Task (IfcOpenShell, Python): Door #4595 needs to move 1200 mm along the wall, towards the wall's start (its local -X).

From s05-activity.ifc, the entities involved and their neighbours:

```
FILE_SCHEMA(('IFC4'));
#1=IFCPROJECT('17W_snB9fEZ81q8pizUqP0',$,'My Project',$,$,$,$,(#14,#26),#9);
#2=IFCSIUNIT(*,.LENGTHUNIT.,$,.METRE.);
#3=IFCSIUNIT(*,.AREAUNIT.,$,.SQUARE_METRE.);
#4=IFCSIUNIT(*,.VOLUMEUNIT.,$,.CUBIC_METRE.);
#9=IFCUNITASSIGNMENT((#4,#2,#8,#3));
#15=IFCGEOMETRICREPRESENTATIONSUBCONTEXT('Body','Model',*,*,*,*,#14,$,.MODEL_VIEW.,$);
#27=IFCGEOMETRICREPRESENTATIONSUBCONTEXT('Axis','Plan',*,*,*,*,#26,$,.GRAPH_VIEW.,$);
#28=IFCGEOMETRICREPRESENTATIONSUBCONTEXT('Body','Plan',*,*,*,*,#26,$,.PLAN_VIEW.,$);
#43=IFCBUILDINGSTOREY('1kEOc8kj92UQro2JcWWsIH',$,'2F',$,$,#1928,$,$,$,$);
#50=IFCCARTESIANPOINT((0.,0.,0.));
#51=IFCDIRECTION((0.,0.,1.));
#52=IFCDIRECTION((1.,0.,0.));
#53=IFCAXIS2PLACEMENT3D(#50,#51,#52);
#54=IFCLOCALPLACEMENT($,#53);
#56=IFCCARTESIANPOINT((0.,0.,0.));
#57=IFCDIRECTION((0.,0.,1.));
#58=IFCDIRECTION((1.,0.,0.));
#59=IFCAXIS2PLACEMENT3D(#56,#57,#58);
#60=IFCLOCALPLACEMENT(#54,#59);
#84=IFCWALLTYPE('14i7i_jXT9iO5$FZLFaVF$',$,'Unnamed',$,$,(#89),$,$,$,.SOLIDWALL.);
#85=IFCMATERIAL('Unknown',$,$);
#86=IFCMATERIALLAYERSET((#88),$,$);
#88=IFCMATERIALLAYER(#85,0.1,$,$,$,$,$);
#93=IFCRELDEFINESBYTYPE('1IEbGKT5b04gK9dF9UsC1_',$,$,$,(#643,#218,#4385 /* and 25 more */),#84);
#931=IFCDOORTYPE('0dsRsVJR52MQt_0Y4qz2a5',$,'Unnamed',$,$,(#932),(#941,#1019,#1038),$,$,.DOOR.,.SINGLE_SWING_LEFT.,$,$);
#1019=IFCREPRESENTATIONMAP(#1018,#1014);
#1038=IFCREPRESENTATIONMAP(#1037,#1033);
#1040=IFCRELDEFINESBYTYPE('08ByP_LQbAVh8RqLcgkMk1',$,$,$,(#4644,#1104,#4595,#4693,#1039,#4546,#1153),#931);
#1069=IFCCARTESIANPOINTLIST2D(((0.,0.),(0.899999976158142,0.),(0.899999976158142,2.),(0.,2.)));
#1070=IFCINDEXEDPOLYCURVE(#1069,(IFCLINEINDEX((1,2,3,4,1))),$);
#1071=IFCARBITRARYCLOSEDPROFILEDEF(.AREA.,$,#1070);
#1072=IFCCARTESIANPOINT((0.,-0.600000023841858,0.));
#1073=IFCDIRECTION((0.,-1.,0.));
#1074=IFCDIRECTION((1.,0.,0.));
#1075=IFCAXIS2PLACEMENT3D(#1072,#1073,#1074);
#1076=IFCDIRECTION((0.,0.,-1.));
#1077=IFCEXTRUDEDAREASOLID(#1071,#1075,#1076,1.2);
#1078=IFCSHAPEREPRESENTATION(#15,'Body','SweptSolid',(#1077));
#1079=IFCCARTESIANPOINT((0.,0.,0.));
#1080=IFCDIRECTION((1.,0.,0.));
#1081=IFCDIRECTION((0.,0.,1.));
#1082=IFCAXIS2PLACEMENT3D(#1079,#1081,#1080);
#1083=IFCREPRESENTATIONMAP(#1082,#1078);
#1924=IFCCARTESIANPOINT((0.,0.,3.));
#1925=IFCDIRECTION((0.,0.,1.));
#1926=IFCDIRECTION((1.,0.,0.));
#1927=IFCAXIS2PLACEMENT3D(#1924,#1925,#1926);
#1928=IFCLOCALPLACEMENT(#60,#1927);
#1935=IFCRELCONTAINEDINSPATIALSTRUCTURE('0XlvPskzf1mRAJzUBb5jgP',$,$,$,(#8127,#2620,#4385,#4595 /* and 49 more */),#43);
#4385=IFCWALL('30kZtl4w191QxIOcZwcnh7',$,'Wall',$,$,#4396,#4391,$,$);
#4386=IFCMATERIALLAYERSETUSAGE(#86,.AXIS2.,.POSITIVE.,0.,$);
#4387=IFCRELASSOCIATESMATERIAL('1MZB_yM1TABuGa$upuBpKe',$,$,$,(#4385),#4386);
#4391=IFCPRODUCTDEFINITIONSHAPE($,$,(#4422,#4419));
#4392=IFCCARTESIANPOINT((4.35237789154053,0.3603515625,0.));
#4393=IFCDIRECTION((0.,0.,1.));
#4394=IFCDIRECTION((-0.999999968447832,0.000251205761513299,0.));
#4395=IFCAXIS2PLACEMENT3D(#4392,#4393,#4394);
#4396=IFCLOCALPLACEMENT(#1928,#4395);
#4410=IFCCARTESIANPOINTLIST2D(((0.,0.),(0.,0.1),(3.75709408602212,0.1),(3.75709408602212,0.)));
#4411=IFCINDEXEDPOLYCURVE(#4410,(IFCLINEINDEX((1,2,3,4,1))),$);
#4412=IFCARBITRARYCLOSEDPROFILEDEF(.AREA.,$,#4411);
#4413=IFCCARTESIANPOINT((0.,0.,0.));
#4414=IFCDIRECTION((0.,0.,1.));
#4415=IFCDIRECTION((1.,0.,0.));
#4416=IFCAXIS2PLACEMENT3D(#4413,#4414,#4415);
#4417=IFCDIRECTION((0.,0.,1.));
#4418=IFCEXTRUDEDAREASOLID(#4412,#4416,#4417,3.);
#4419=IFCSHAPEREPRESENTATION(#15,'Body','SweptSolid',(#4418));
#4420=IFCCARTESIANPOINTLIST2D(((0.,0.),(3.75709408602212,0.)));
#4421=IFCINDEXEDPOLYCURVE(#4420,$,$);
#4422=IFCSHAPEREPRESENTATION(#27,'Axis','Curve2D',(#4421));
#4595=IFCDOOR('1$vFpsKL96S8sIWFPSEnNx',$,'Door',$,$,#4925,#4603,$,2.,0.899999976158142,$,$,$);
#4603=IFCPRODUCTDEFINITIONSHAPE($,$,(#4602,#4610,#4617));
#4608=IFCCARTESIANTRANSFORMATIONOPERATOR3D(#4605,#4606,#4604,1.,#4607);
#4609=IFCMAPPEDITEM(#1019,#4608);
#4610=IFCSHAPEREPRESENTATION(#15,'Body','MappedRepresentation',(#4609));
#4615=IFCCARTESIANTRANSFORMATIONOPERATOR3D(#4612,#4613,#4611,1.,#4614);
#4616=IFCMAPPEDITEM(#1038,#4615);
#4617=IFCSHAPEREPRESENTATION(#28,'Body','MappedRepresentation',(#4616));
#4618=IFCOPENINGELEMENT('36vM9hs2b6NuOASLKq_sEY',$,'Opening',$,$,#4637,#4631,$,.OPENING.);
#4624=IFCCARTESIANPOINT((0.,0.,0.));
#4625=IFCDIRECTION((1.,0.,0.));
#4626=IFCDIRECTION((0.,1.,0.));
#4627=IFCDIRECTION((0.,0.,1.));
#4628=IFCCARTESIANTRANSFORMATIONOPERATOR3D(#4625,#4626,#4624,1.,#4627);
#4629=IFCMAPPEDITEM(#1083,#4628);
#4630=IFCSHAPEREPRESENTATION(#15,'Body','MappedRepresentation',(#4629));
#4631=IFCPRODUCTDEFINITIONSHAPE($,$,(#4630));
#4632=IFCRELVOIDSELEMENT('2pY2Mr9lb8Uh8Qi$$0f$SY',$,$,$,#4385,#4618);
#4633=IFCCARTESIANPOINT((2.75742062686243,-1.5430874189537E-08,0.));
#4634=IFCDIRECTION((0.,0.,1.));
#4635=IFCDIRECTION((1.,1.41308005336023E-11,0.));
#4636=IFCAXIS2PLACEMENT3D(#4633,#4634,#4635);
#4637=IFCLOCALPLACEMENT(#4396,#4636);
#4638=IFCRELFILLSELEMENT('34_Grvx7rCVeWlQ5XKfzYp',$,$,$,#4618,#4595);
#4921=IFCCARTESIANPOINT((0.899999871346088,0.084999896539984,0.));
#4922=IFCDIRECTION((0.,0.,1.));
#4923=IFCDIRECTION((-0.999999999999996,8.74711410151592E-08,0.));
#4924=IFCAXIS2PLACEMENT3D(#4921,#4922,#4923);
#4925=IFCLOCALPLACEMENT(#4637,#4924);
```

```python
import ifcopenshell
import ifcopenshell.api.geometry
import ifcopenshell.util.placement
import ifcopenshell.util.unit

model = ifcopenshell.open("s05-activity.ifc")
unit_scale = ifcopenshell.util.unit.calculate_unit_scale(model)

door = model.by_guid("1$vFpsKL96S8sIWFPSEnNx")
opening = door.FillsVoids[0].RelatingOpeningElement
wall = opening.VoidsElements[0].RelatingBuildingElement

wall_matrix = ifcopenshell.util.placement.get_local_placement(wall.ObjectPlacement)
shift = wall_matrix[:3, 0] * -1.2 / unit_scale
before = ifcopenshell.util.placement.get_local_placement(door.ObjectPlacement)[:3, 3].copy()

# The door is placed relative to its opening, so it follows when the opening moves.
matrix = ifcopenshell.util.placement.get_local_placement(opening.ObjectPlacement)
matrix[:3, 3] += shift
ifcopenshell.api.geometry.edit_object_placement(
    model, product=opening, matrix=matrix, is_si=False, should_transform_children=True
)

after = ifcopenshell.util.placement.get_local_placement(door.ObjectPlacement)[:3, 3]
print("door moved by", (after - before).round(3) + 0.0)

model.write("s05-activity_edited.ifc")
```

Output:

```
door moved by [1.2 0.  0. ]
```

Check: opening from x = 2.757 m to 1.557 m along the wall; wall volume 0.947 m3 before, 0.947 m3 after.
